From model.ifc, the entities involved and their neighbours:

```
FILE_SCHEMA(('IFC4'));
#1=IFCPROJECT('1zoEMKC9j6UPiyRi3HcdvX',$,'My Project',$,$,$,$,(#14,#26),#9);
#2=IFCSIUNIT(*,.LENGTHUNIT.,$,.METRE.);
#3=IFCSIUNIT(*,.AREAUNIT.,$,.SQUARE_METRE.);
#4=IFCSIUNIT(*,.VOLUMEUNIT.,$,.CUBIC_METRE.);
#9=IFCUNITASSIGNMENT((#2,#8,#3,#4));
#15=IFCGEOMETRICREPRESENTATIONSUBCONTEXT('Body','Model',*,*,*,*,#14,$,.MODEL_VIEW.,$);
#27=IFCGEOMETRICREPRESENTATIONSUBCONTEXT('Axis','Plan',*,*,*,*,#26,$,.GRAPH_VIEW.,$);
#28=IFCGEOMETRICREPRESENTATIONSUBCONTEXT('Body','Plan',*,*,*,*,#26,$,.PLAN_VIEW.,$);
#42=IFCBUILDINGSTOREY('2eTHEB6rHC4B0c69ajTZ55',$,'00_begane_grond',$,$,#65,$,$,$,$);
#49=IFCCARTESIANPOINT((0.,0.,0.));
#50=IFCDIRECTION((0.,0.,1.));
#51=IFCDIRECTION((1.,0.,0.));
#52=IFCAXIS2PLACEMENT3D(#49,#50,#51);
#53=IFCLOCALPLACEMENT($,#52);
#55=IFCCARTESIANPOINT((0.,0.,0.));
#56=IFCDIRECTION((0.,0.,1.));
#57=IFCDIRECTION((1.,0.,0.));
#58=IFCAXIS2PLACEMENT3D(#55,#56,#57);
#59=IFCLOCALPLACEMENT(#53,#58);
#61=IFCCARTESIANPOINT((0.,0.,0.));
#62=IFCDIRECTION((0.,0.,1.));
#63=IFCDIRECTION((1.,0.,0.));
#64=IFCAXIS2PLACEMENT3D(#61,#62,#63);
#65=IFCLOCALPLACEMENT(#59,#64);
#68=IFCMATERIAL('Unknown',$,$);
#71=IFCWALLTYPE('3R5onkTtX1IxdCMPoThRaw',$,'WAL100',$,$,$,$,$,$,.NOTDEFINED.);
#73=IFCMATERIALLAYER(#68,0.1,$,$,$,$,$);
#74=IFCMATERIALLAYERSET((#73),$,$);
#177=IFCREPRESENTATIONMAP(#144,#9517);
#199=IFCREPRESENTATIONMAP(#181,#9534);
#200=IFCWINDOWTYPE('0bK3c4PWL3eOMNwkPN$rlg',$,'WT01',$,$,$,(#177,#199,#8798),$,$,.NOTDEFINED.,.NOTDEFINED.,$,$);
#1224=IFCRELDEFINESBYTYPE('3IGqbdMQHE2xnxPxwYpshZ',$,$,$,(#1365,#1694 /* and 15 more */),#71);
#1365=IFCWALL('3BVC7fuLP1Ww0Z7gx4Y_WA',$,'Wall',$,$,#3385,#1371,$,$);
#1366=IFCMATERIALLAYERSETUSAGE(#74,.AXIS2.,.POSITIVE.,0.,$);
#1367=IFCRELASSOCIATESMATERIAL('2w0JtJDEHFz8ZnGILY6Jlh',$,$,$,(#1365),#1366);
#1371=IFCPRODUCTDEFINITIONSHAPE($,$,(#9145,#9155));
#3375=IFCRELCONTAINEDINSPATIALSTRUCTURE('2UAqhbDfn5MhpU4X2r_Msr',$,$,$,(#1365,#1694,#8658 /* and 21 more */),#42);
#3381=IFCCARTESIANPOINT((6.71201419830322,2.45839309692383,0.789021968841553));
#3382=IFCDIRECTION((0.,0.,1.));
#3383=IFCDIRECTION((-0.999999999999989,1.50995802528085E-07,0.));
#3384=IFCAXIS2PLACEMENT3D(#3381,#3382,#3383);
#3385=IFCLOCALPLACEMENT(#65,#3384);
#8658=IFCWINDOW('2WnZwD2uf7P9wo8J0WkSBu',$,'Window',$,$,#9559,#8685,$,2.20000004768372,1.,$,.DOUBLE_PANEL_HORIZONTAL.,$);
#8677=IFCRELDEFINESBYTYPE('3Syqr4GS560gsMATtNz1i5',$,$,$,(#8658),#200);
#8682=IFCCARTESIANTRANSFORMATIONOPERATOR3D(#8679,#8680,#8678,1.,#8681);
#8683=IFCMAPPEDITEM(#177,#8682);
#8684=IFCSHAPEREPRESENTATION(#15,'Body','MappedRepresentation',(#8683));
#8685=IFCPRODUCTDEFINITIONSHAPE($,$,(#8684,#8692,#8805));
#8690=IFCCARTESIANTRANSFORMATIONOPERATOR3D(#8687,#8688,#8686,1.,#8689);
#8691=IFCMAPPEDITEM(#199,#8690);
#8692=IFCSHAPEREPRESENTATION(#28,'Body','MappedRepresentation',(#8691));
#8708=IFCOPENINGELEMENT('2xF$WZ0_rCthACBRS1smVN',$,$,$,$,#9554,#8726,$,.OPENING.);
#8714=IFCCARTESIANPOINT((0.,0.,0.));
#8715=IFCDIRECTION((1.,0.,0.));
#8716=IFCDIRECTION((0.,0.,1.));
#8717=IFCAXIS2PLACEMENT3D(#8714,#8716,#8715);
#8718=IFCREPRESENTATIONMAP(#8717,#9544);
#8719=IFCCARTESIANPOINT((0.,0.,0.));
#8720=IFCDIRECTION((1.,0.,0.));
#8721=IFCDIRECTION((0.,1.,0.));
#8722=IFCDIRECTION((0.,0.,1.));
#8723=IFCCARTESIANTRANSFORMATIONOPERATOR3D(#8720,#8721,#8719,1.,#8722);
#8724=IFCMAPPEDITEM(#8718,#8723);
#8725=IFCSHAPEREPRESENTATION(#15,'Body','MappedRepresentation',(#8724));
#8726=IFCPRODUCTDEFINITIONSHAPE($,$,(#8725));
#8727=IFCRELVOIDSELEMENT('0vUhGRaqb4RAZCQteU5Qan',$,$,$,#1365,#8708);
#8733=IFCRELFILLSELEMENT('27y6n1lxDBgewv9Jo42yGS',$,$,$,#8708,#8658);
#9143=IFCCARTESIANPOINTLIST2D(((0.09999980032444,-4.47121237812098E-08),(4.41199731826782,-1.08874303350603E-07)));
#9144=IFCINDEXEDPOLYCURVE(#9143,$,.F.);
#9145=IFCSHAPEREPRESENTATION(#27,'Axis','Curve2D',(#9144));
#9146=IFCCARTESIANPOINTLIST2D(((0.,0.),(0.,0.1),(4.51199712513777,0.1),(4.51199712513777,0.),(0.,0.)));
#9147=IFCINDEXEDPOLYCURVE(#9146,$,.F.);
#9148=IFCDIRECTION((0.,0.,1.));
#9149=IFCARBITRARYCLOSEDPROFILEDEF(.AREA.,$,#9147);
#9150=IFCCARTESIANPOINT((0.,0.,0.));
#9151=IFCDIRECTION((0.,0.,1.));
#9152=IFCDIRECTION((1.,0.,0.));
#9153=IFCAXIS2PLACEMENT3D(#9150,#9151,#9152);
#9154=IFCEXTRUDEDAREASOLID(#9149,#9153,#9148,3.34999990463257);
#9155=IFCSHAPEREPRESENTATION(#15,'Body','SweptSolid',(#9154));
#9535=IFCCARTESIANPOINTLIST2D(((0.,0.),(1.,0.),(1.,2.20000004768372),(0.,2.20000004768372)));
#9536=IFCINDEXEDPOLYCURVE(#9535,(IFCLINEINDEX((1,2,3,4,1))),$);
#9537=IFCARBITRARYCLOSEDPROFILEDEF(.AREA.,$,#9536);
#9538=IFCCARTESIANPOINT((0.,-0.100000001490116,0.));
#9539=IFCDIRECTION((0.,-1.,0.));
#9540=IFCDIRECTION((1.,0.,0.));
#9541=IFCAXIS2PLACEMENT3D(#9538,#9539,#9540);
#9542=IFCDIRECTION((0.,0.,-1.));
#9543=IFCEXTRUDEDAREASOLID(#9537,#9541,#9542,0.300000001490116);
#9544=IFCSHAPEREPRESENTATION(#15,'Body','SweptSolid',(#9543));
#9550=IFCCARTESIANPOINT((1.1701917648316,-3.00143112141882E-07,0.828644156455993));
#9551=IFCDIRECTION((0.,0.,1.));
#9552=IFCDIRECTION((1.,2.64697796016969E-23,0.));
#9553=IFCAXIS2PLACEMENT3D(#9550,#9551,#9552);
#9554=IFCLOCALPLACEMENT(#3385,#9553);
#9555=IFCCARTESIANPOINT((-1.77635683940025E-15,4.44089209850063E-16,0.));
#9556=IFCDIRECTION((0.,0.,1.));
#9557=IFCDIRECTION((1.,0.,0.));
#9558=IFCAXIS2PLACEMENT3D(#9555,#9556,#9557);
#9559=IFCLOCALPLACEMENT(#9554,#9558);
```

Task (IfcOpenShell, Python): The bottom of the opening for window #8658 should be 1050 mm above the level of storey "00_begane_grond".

```python
import numpy as np
import ifcopenshell
import ifcopenshell.api.geometry
import ifcopenshell.geom
import ifcopenshell.util.element
import ifcopenshell.util.placement
import ifcopenshell.util.shape
import ifcopenshell.util.unit

model = ifcopenshell.open("model.ifc")
unit_scale = ifcopenshell.util.unit.calculate_unit_scale(model)

window = model.by_guid("2WnZwD2uf7P9wo8J0WkSBu")
opening = window.FillsVoids[0].RelatingOpeningElement
storey = ifcopenshell.util.element.get_container(window, ifc_class="IfcBuildingStorey")
level = ifcopenshell.util.placement.get_local_placement(storey.ObjectPlacement)[2, 3]

# The opening's origin need not be at the sill, so measure its lowest point.
shape = ifcopenshell.geom.create_shape(ifcopenshell.geom.settings(), opening)
bottom = ifcopenshell.util.shape.get_shape_bottom_elevation(shape, shape.geometry) / unit_scale
dz = level + 1.05 / unit_scale - bottom

shift = np.array([0.0, 0.0, dz])
# The window is placed relative to its opening, so it follows when the opening moves.
matrix = ifcopenshell.util.placement.get_local_placement(opening.ObjectPlacement)
matrix[:3, 3] += shift
ifcopenshell.api.geometry.edit_object_placement(
    model, product=opening, matrix=matrix, is_si=False, should_transform_children=True
)

print(f"moved by {dz * unit_scale:+.3f} m")

model.write("model_edited.ifc")
```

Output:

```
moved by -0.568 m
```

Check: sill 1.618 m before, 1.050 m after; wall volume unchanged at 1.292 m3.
